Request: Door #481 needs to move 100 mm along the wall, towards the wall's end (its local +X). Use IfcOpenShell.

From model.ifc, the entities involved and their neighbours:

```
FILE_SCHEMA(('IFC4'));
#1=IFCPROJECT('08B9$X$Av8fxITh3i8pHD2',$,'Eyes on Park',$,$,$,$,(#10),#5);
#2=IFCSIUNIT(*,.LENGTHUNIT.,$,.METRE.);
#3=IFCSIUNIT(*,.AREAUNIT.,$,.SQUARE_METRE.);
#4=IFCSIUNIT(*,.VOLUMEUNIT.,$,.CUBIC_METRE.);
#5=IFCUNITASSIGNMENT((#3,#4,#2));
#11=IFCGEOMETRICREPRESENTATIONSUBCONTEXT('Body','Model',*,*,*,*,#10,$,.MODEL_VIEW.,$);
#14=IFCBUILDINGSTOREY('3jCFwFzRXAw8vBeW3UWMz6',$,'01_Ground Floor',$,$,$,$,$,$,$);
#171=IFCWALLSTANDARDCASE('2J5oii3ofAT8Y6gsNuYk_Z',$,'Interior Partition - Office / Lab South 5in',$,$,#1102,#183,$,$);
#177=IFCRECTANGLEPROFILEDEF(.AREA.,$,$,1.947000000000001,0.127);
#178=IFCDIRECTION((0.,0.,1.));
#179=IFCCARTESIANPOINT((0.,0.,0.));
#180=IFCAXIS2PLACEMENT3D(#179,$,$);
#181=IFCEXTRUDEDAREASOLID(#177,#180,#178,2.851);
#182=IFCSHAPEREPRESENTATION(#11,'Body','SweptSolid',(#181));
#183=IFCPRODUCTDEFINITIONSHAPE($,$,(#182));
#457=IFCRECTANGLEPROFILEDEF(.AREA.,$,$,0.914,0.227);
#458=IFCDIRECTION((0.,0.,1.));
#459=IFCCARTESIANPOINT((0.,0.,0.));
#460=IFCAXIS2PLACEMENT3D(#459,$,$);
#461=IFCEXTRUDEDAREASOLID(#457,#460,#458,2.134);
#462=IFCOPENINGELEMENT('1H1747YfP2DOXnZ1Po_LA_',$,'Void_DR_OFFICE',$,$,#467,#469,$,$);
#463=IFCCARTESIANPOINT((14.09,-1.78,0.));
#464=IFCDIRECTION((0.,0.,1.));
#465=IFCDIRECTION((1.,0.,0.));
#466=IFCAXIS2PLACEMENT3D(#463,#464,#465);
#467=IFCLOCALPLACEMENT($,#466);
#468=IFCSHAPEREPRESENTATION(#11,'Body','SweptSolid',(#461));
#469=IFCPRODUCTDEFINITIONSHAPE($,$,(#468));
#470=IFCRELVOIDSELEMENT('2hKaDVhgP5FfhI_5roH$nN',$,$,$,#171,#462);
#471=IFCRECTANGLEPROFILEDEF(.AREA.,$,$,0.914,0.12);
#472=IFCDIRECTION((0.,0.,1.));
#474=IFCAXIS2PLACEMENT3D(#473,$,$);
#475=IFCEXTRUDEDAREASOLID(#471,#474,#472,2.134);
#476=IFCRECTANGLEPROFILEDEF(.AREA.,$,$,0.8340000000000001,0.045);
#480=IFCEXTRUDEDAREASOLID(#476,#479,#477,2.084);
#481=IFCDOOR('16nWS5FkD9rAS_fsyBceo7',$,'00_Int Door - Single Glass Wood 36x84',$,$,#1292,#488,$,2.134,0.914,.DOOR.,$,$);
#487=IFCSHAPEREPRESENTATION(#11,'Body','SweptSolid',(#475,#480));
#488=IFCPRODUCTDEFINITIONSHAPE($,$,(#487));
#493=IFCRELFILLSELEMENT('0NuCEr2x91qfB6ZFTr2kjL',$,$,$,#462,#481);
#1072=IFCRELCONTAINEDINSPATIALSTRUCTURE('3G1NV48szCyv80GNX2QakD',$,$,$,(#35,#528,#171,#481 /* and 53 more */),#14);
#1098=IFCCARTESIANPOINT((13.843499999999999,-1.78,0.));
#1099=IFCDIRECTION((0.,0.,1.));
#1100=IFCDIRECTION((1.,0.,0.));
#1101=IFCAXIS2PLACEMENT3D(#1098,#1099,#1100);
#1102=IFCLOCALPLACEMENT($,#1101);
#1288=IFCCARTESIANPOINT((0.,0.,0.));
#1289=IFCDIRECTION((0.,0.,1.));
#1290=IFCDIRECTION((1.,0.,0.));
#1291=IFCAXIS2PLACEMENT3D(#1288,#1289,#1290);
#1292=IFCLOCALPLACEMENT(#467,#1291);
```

```python
import ifcopenshell
import ifcopenshell.api.geometry
import ifcopenshell.util.placement

model = ifcopenshell.open("model.ifc")

door = model.by_guid("16nWS5FkD9rAS_fsyBceo7")
opening = door.FillsVoids[0].RelatingOpeningElement
wall = opening.VoidsElements[0].RelatingBuildingElement

wall_matrix = ifcopenshell.util.placement.get_local_placement(wall.ObjectPlacement)
shift = wall_matrix[:3, 0] * 0.1
before = ifcopenshell.util.placement.get_local_placement(door.ObjectPlacement)[:3, 3].copy()

# The door is placed relative to its opening, so it follows when the opening moves.
matrix = ifcopenshell.util.placement.get_local_placement(opening.ObjectPlacement)
matrix[:3, 3] += shift
ifcopenshell.api.geometry.edit_object_placement(
    model, product=opening, matrix=matrix, is_si=False, should_transform_children=True
)

after = ifcopenshell.util.placement.get_local_placement(door.ObjectPlacement)[:3, 3]
print("door moved by", (after - before).round(3) + 0.0)

model.write("model_updated.ifc")
```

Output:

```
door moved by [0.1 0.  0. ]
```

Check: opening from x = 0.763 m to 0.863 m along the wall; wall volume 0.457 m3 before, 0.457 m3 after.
